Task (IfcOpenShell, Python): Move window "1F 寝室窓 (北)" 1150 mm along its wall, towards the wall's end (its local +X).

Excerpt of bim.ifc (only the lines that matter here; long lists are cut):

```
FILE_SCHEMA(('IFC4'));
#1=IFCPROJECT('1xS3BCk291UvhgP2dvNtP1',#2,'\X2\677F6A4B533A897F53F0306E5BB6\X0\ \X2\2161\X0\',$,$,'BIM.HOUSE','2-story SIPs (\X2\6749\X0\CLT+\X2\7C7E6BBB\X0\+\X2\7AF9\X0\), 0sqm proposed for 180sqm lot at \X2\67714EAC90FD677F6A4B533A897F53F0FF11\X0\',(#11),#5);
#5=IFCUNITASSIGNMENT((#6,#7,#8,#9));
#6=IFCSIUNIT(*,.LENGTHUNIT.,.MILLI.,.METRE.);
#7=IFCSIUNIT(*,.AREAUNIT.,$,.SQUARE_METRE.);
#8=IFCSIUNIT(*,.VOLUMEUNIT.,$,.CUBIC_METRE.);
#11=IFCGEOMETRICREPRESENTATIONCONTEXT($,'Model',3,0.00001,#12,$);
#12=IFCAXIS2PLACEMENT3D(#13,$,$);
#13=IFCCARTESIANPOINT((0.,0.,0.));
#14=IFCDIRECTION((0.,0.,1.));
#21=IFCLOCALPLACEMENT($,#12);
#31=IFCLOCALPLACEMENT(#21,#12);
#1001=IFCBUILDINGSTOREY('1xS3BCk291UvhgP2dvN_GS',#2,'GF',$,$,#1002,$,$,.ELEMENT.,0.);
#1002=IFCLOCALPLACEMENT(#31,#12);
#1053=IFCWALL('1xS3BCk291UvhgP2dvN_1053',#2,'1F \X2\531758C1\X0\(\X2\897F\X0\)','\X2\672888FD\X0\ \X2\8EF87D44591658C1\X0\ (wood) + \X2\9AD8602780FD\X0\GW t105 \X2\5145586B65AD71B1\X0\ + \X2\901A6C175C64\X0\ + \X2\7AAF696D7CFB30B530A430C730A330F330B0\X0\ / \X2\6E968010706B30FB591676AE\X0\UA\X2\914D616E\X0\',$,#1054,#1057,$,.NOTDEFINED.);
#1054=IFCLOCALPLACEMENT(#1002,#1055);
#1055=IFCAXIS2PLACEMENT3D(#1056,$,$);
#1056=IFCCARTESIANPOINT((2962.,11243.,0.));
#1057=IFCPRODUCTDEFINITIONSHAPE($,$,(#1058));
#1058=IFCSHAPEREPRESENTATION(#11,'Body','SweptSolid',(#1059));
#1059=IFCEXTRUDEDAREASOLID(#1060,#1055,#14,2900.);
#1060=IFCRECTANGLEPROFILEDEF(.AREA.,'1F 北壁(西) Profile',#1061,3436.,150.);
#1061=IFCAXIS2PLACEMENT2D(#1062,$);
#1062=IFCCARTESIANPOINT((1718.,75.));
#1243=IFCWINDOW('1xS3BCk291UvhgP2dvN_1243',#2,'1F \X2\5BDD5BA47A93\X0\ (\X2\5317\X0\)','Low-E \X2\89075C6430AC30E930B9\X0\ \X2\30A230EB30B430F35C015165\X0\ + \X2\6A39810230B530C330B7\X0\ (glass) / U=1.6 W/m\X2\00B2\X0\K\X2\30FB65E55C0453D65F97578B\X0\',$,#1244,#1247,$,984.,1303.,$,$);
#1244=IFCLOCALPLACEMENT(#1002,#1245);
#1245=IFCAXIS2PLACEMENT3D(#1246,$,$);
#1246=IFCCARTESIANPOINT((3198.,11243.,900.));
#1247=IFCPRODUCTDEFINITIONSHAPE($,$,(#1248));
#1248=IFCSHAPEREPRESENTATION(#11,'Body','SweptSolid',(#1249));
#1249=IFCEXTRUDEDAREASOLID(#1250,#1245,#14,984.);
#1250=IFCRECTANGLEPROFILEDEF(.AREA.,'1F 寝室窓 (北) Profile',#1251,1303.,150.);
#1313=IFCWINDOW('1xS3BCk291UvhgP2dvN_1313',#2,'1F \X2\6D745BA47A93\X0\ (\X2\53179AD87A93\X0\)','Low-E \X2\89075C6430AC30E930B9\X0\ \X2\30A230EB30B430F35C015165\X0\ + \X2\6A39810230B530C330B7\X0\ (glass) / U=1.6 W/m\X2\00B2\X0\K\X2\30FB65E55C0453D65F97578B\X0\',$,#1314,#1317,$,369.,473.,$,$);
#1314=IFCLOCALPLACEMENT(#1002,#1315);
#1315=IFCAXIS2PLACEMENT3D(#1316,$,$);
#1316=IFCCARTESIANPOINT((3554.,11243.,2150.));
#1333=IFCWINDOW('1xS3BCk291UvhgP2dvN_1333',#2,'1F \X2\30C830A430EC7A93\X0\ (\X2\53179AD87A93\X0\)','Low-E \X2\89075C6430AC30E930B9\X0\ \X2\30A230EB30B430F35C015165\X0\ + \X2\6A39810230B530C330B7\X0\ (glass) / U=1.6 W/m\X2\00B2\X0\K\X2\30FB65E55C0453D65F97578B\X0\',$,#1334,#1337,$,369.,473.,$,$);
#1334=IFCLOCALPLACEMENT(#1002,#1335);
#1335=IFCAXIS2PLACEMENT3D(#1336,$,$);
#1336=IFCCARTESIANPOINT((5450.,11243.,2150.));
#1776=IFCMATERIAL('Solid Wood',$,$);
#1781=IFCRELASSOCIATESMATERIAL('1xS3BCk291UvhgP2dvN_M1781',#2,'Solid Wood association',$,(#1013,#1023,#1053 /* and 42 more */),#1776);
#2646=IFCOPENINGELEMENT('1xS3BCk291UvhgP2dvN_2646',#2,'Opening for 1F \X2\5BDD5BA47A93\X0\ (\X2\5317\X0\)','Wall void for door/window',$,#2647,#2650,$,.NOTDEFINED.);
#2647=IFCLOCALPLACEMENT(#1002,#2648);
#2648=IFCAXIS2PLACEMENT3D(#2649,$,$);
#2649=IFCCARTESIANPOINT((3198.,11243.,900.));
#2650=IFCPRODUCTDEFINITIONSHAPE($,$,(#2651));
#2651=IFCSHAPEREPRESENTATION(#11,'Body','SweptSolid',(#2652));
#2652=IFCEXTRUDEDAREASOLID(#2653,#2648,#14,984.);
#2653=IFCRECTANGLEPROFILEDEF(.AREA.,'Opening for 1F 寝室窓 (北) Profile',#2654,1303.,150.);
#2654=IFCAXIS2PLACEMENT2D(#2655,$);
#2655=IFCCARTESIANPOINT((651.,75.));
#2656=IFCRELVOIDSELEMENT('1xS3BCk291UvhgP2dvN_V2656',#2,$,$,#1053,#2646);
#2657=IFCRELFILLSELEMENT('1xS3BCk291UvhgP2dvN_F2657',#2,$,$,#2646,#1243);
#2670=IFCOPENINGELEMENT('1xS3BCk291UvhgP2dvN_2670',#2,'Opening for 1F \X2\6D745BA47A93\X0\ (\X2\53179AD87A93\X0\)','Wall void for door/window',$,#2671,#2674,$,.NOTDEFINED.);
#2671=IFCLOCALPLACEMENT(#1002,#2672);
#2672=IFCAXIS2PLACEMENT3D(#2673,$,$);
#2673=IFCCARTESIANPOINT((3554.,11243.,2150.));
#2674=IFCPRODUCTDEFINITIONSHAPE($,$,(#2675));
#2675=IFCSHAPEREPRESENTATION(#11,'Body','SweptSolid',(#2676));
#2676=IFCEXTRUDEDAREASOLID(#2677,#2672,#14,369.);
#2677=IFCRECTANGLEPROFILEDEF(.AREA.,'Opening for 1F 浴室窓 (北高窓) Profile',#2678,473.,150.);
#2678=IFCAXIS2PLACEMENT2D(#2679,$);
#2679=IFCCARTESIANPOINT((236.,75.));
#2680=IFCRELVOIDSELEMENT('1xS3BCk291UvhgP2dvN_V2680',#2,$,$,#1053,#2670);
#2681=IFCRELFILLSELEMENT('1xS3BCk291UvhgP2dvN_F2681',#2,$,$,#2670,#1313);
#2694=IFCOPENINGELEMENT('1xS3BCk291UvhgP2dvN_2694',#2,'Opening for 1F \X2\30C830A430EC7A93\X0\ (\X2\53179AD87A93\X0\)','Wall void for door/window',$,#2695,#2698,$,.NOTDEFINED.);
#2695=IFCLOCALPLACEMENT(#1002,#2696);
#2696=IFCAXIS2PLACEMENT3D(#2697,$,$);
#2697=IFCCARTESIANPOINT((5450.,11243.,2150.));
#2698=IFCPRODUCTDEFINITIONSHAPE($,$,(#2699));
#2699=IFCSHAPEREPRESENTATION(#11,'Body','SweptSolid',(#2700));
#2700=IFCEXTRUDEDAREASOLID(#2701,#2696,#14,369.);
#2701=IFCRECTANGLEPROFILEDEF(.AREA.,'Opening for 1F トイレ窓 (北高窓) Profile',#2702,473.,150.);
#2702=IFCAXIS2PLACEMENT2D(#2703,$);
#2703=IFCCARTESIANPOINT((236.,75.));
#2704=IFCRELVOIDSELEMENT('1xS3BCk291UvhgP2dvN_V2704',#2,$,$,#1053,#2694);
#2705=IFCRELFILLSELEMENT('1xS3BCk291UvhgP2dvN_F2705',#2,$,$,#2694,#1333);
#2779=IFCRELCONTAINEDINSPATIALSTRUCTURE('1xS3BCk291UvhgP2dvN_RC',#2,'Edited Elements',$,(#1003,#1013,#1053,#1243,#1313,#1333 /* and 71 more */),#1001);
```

```python
import ifcopenshell
import ifcopenshell.api.geometry
import ifcopenshell.util.placement
import ifcopenshell.util.unit

model = ifcopenshell.open("bim.ifc")
unit_scale = ifcopenshell.util.unit.calculate_unit_scale(model)

window = model.by_guid("1xS3BCk291UvhgP2dvN_1243")
opening = window.FillsVoids[0].RelatingOpeningElement
wall = opening.VoidsElements[0].RelatingBuildingElement

wall_matrix = ifcopenshell.util.placement.get_local_placement(wall.ObjectPlacement)
shift = wall_matrix[:3, 0] * 1.15 / unit_scale
before = ifcopenshell.util.placement.get_local_placement(window.ObjectPlacement)[:3, 3].copy()

# The window is not placed relative to its opening, so move both.
for product in (opening, window):
    matrix = ifcopenshell.util.placement.get_local_placement(product.ObjectPlacement)
    matrix[:3, 3] += shift
    ifcopenshell.api.geometry.edit_object_placement(model, product=product, matrix=matrix, is_si=False)

after = ifcopenshell.util.placement.get_local_placement(window.ObjectPlacement)[:3, 3]
print("window moved by", (after - before).round(3) + 0.0)

model.write("bim_updated.ifc")
```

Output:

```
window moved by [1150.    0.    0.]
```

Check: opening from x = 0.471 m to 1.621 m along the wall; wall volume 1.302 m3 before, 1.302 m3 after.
